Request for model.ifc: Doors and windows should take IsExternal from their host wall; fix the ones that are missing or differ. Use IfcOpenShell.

First a look at what the model holds.

```python
import ifcopenshell
import ifcopenshell.util.element

model = ifcopenshell.open("model.ifc")
print(model.schema)
seen = {}
for e in model.by_type("IfcDoor") + model.by_type("IfcWindow"):
    if not e.FillsVoids:
        continue
    host = e.FillsVoids[0].RelatingOpeningElement.VoidsElements[0].RelatingBuildingElement
    own = ifcopenshell.util.element.get_pset(e, f"Pset_{e.is_a()[3:].removesuffix('StandardCase')}Common", "IsExternal")
    wall = ifcopenshell.util.element.get_pset(host, "Pset_WallCommon", "IsExternal")
    seen[e.is_a(), own, wall] = seen.get((e.is_a(), own, wall), 0) + 1
for (cls, own, wall), count in sorted(seen.items(), key=str):
    print(count, cls, "IsExternal:", own, "| host wall:", wall)
```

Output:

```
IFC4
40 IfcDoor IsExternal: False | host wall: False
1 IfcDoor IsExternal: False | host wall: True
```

```python
import ifcopenshell
import ifcopenshell.api.pset
import ifcopenshell.util.element

model = ifcopenshell.open("model.ifc")

count = 0
for ifc_class, pset_name in (("IfcDoor", "Pset_DoorCommon"), ("IfcWindow", "Pset_WindowCommon")):
    for e in model.by_type(ifc_class):
        if not e.FillsVoids:
            continue
        host = e.FillsVoids[0].RelatingOpeningElement.VoidsElements[0].RelatingBuildingElement
        external = ifcopenshell.util.element.get_pset(host, "Pset_WallCommon", "IsExternal")
        if external is None or ifcopenshell.util.element.get_pset(e, pset_name, "IsExternal") == external:
            continue
        pset = ifcopenshell.api.pset.add_pset(model, product=e, name=pset_name)
        ifcopenshell.api.pset.edit_pset(model, pset=pset, properties={"IsExternal": external})
        count += 1

print(count, "updated")

model.write("model_rev.ifc")
```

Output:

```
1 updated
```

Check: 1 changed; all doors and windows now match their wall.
